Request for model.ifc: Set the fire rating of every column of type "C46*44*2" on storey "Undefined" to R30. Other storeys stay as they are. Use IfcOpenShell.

First a look at what the model holds.

```python
import ifcopenshell
import ifcopenshell.util.element

model = ifcopenshell.open("model.ifc")
print(model.schema)
storey = next(s for s in model.by_type("IfcBuildingStorey") if s.Name == "Undefined")
columns = [e for e in ifcopenshell.util.element.get_decomposition(storey) if e.is_a("IfcColumn")]
seen = {}
for e in columns:
    element_type = ifcopenshell.util.element.get_type(e)
    key = (element_type.Name if element_type != e and element_type else None, ifcopenshell.util.element.get_pset(e, "Pset_ColumnCommon", "FireRating"))
    seen[key] = seen.get(key, 0) + 1
for (name, value), count in sorted(seen.items(), key=str):
    print(count, "x", name, "|", value)
```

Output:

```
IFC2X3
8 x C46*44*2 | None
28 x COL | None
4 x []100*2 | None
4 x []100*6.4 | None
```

```python
import ifcopenshell
import ifcopenshell.api.pset
import ifcopenshell.util.element

model = ifcopenshell.open("model.ifc")

storey = next(s for s in model.by_type("IfcBuildingStorey") if s.Name == "Undefined")
columns = [e for e in ifcopenshell.util.element.get_decomposition(storey) if e.is_a("IfcColumn")]

count = 0
for e in columns:
    element_type = ifcopenshell.util.element.get_type(e)
    if element_type in (None, e) or element_type.Name != "C46*44*2":
        continue
    found = ifcopenshell.util.element.get_pset(e, "Pset_ColumnCommon", should_inherit=False)
    if found:
        pset = model.by_id(found["id"])
        if len(ifcopenshell.util.element.get_elements_by_pset(pset)) > 1:
            pset = ifcopenshell.api.pset.unshare_pset(model, products=[e], pset=pset)[0]
    else:
        pset = ifcopenshell.api.pset.add_pset(model, product=e, name="Pset_ColumnCommon")
    ifcopenshell.api.pset.edit_pset(model, pset=pset, properties={"FireRating": "R30"})
    count += 1

print(count, "columns updated")

model.write("model_updated.ifc")
```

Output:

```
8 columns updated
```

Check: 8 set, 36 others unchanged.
